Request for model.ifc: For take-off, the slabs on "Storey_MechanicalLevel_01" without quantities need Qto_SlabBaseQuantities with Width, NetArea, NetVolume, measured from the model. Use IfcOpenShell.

First a look at what the model holds.

```python
import ifcopenshell
import ifcopenshell.util.element
import ifcopenshell.util.unit

model = ifcopenshell.open("model.ifc")
print(model.schema)
for unit_type in ("LENGTHUNIT", "AREAUNIT", "VOLUMEUNIT"):
    print(unit_type, ifcopenshell.util.unit.calculate_unit_scale(model, unit_type))
storey = next(s for s in model.by_type("IfcBuildingStorey") if s.Name == "Storey_MechanicalLevel_01")
slabs = [e for e in ifcopenshell.util.element.get_decomposition(storey) if e.is_a("IfcSlab")]
for e in sorted(slabs, key=lambda e: e.id()):
    print(e.id(), e.is_a(), e.Name, list(ifcopenshell.util.element.get_psets(e, qtos_only=True)), sep=" | ")
```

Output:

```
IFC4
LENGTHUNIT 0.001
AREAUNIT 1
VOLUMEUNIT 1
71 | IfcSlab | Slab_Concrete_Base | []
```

```python
import ifcopenshell
import ifcopenshell.api.pset
import ifcopenshell.geom
import ifcopenshell.util.element
import ifcopenshell.util.shape
import ifcopenshell.util.unit

model = ifcopenshell.open("model.ifc")
unit_scale = ifcopenshell.util.unit.calculate_unit_scale(model)
area_scale = ifcopenshell.util.unit.calculate_unit_scale(model, "AREAUNIT")
volume_scale = ifcopenshell.util.unit.calculate_unit_scale(model, "VOLUMEUNIT")
settings = ifcopenshell.geom.settings()

storey = next(s for s in model.by_type("IfcBuildingStorey") if s.Name == "Storey_MechanicalLevel_01")
slabs = [e for e in ifcopenshell.util.element.get_decomposition(storey) if e.is_a("IfcSlab")]

for e in sorted(slabs, key=lambda e: e.id()):
    if ifcopenshell.util.element.get_psets(e, qtos_only=True, should_inherit=False):
        continue
    # Geometry comes back in metres, in the element's own axes.
    shape = ifcopenshell.geom.create_shape(settings, e)
    values = {
        "Width": ifcopenshell.util.shape.get_z(shape.geometry) / unit_scale,
        "NetArea": ifcopenshell.util.shape.get_footprint_area(shape.geometry) / area_scale,
        "NetVolume": ifcopenshell.util.shape.get_volume(shape.geometry) / volume_scale,
    }
    qto = ifcopenshell.api.pset.add_qto(model, product=e, name="Qto_SlabBaseQuantities")
    ifcopenshell.api.pset.edit_qto(model, qto=qto, properties=values)
    print(e.id(), {k: round(v, 3) for k, v in values.items()})

model.write("model_v2.ifc")
```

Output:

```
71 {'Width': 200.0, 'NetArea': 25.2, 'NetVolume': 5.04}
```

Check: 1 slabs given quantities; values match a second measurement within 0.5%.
